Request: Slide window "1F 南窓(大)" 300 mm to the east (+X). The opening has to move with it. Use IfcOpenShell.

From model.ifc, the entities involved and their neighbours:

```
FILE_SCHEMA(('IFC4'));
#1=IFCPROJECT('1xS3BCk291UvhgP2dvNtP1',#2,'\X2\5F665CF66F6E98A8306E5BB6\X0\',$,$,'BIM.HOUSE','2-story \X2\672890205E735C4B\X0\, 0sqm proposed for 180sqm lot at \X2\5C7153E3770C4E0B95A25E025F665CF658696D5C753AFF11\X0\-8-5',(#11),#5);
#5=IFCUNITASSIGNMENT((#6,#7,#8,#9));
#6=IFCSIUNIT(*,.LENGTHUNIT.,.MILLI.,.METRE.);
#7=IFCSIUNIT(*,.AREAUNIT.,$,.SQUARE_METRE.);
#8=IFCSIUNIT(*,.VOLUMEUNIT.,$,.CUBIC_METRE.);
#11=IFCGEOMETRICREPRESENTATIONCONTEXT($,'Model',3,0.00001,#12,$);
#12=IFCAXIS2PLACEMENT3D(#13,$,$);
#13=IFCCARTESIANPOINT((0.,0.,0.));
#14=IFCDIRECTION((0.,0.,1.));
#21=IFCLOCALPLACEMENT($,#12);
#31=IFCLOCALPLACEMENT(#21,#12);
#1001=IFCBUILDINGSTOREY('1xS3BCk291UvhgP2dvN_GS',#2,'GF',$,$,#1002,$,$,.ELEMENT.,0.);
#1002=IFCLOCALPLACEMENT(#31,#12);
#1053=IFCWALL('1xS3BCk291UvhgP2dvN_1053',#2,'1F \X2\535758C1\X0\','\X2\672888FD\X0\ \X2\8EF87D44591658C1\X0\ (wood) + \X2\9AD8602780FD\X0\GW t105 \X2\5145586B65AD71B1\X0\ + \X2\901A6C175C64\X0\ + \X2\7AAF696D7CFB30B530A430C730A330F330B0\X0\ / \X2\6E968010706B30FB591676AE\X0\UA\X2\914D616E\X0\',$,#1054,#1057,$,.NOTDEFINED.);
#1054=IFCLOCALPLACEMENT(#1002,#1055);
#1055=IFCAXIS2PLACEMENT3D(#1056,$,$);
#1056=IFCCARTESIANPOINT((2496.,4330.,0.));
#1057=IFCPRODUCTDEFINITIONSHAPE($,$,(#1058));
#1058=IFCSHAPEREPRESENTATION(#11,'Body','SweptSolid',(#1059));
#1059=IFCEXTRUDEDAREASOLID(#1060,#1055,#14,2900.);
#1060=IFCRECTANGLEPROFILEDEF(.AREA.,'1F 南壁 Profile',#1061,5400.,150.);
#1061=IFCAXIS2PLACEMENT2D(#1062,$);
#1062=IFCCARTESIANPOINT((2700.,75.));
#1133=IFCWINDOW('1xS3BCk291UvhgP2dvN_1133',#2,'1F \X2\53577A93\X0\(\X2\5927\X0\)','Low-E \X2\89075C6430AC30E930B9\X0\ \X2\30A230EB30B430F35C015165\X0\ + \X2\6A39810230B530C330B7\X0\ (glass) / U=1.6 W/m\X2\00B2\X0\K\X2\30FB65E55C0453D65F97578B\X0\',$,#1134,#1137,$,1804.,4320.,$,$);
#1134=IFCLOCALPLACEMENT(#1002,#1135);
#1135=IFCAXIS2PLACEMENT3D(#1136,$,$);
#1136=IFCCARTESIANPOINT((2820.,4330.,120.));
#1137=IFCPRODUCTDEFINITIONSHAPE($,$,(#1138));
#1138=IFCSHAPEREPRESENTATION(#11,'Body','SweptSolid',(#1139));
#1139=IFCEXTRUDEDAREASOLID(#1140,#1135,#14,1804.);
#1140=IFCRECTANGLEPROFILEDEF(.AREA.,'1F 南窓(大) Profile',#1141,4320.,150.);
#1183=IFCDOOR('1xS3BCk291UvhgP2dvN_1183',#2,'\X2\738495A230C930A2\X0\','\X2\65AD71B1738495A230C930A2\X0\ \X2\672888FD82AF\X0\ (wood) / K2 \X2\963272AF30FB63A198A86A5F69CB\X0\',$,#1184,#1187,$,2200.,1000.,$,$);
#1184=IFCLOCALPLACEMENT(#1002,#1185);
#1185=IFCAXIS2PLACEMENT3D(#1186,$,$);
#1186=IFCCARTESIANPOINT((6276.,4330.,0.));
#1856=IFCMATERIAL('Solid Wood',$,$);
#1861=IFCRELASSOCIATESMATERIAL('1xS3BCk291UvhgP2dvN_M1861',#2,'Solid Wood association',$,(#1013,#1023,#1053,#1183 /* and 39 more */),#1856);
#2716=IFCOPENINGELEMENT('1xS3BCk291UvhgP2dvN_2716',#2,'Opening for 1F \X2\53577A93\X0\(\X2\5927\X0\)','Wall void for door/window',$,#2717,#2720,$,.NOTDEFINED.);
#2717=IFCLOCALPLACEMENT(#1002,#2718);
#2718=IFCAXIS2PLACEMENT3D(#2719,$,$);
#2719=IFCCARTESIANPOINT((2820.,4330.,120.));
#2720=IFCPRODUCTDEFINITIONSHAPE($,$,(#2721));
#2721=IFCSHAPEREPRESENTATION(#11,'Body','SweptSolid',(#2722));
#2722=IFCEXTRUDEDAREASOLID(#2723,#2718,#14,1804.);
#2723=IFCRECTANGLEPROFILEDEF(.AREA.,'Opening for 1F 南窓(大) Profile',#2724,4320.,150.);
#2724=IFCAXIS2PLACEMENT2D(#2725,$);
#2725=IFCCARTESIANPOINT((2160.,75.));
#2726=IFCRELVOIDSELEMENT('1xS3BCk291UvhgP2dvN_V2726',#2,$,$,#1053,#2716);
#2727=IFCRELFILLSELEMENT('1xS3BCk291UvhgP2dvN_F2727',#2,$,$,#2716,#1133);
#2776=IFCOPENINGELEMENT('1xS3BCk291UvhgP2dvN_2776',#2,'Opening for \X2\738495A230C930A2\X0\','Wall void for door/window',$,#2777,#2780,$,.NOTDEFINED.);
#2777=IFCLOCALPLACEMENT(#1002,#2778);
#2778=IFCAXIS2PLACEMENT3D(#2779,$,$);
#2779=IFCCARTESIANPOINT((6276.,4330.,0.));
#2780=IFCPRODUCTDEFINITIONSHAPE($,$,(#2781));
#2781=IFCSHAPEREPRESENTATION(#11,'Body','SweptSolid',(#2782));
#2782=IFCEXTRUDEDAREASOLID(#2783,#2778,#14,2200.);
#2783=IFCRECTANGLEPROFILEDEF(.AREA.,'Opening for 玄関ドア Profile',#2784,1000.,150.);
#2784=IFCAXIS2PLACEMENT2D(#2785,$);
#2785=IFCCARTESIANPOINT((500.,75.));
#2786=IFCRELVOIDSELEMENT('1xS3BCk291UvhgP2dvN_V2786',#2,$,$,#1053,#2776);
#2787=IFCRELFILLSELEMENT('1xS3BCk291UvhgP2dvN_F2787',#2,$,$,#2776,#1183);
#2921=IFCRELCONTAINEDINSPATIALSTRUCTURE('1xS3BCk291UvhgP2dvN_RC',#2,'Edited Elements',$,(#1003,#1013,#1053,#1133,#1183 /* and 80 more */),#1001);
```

```python
import ifcopenshell
import ifcopenshell.api.geometry
import ifcopenshell.util.placement

model = ifcopenshell.open("model.ifc")

window = model.by_id(1133)
opening = window.FillsVoids[0].RelatingOpeningElement
wall = opening.VoidsElements[0].RelatingBuildingElement

wall_matrix = ifcopenshell.util.placement.get_local_placement(wall.ObjectPlacement)
shift = wall_matrix[:3, 0] * 300.0
before = ifcopenshell.util.placement.get_local_placement(window.ObjectPlacement)[:3, 3].copy()

# The window is not placed relative to its opening, so move both.
for product in (opening, window):
    matrix = ifcopenshell.util.placement.get_local_placement(product.ObjectPlacement)
    matrix[:3, 3] += shift
    ifcopenshell.api.geometry.edit_object_placement(model, product=product, matrix=matrix, is_si=False)

after = ifcopenshell.util.placement.get_local_placement(window.ObjectPlacement)[:3, 3]
print("window moved by", (after - before).round(3) + 0.0)

model.write("model_rev.ifc")
```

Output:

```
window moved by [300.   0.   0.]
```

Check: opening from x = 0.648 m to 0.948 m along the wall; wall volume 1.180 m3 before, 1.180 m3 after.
